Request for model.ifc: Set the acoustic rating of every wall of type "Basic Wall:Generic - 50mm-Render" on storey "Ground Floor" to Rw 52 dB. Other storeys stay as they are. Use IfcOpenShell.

First a look at what the model holds.

```python
import ifcopenshell
import ifcopenshell.util.element

model = ifcopenshell.open("model.ifc")
print(model.schema)
storey = next(s for s in model.by_type("IfcBuildingStorey") if s.Name == "Ground Floor")
walls = [e for e in ifcopenshell.util.element.get_decomposition(storey) if e.is_a("IfcWall")]
seen = {}
for e in walls:
    element_type = ifcopenshell.util.element.get_type(e)
    key = (element_type.Name if element_type != e and element_type else None, ifcopenshell.util.element.get_pset(e, "Pset_WallCommon", "AcousticRating"))
    seen[key] = seen.get(key, 0) + 1
for (name, value), count in sorted(seen.items(), key=str):
    print(count, "x", name, "|", value)
```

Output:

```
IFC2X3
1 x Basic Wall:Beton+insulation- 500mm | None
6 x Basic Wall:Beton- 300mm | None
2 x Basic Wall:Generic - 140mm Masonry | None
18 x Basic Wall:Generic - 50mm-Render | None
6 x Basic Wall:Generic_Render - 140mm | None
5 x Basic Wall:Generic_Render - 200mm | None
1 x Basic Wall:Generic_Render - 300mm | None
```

```python
import ifcopenshell
import ifcopenshell.api.pset
import ifcopenshell.util.element

model = ifcopenshell.open("model.ifc")

storey = next(s for s in model.by_type("IfcBuildingStorey") if s.Name == "Ground Floor")
walls = [e for e in ifcopenshell.util.element.get_decomposition(storey) if e.is_a("IfcWall")]

count = 0
for e in walls:
    element_type = ifcopenshell.util.element.get_type(e)
    if element_type in (None, e) or element_type.Name != "Basic Wall:Generic - 50mm-Render":
        continue
    # add_pset returns the element's existing set when there is one.
    pset = ifcopenshell.api.pset.add_pset(model, product=e, name="Pset_WallCommon")
    ifcopenshell.api.pset.edit_pset(model, pset=pset, properties={"AcousticRating": "Rw 52 dB"})
    count += 1

print(count, "walls updated")

model.write("model_v2.ifc")
```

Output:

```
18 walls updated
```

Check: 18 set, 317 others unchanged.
